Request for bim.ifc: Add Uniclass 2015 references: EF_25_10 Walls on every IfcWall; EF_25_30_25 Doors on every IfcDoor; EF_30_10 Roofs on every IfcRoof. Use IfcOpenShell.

First a look at what the model holds.

```python
import ifcopenshell

model = ifcopenshell.open("bim.ifc")
print(model.schema)
print("classifications:", [c.Name for c in model.by_type("IfcClassification")])
for ifc_class in ("IfcDoor", "IfcRoof", "IfcStair", "IfcWall", "IfcWindow"):
    print(ifc_class, len(model.by_type(ifc_class)))
```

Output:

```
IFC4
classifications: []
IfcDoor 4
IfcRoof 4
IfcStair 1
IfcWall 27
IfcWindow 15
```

```python
import ifcopenshell
import ifcopenshell.api.classification

model = ifcopenshell.open("bim.ifc")

system = ifcopenshell.api.classification.add_classification(model, classification="Uniclass 2015")

codes = {
    "IfcWall": ("EF_25_10", "Walls"),
    "IfcDoor": ("EF_25_30_25", "Doors"),
    "IfcRoof": ("EF_30_10", "Roofs"),
}
for ifc_class, (code, name) in codes.items():
    products = model.by_type(ifc_class)
    ifcopenshell.api.classification.add_reference(
        model, products=products, classification=system, identification=code, name=name
    )
    print(code, len(products))

model.write("bim_updated.ifc")
```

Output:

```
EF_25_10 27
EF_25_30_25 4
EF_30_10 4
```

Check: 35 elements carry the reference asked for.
